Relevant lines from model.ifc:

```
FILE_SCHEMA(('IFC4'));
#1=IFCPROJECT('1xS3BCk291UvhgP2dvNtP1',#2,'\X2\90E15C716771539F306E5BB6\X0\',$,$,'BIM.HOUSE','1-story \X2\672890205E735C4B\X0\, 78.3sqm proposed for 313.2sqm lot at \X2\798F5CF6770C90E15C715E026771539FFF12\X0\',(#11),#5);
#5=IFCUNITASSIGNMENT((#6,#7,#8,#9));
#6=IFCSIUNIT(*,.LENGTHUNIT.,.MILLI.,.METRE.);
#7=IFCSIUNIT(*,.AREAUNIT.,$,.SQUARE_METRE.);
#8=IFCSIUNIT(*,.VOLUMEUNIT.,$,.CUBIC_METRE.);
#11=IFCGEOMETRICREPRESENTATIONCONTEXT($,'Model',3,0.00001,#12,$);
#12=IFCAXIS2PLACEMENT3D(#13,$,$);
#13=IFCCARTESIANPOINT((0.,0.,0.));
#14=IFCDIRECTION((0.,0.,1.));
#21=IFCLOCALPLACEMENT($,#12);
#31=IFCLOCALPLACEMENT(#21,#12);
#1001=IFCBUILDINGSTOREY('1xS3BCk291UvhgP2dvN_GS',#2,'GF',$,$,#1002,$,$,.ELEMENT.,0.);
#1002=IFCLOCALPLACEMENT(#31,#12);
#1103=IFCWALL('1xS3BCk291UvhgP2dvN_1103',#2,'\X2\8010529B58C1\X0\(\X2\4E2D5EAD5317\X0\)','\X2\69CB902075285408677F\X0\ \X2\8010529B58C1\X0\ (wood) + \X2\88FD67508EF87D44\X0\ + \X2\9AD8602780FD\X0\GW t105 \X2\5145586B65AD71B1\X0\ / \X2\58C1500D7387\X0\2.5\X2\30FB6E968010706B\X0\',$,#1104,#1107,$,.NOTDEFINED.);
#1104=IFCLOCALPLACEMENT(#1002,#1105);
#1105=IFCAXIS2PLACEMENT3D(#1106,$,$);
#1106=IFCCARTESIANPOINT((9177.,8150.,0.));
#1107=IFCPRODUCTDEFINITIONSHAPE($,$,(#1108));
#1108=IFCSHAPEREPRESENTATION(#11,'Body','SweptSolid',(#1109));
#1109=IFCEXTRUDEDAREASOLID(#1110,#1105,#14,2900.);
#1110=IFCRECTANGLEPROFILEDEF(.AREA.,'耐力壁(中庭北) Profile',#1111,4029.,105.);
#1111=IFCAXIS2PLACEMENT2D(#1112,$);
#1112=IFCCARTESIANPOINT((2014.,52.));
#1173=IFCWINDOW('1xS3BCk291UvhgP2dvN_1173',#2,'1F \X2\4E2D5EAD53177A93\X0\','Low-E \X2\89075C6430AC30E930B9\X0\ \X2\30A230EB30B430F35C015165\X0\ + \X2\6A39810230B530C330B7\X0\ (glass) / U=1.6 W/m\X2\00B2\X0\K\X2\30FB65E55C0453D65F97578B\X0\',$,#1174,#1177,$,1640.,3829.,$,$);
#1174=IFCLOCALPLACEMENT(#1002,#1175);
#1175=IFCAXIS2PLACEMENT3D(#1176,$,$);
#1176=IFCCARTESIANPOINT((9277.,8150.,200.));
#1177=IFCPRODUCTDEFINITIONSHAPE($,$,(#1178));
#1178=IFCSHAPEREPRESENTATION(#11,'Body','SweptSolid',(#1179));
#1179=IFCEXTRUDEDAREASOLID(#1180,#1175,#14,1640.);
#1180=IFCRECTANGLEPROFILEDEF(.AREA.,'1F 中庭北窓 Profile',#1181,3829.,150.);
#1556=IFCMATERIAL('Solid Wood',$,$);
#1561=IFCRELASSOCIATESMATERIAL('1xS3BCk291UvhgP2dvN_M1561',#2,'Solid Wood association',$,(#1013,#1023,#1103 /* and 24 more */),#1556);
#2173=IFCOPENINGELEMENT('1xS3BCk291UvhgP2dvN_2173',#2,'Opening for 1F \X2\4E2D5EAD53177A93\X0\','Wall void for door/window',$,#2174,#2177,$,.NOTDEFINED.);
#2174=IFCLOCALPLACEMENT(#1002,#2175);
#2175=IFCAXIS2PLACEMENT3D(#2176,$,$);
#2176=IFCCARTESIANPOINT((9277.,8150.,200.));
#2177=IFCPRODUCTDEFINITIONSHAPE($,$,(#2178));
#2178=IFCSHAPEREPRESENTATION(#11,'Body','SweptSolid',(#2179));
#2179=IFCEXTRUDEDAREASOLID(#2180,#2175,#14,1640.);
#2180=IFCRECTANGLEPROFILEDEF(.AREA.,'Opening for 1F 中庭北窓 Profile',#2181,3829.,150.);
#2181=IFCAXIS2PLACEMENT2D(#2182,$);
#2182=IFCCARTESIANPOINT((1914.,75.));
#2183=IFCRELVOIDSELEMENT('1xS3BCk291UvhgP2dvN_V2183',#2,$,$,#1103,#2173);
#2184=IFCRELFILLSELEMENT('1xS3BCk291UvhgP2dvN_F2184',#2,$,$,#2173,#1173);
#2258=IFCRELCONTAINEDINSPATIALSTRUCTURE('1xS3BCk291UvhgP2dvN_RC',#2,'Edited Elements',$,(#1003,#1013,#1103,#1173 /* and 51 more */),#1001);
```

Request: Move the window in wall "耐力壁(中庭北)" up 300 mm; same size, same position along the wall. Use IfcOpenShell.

```python
import numpy as np
import ifcopenshell
import ifcopenshell.api.geometry
import ifcopenshell.util.placement
import ifcopenshell.util.unit

model = ifcopenshell.open("model.ifc")
unit_scale = ifcopenshell.util.unit.calculate_unit_scale(model)

window = model.by_guid("1xS3BCk291UvhgP2dvN_1173")
opening = window.FillsVoids[0].RelatingOpeningElement
dz = 300.0

shift = np.array([0.0, 0.0, dz])
# The window is not placed relative to its opening, so move both.
for product in (opening, window):
    matrix = ifcopenshell.util.placement.get_local_placement(product.ObjectPlacement)
    matrix[:3, 3] += shift
    ifcopenshell.api.geometry.edit_object_placement(model, product=product, matrix=matrix, is_si=False)

print(f"moved by {dz * unit_scale:+.3f} m")

model.write("model_updated.ifc")
```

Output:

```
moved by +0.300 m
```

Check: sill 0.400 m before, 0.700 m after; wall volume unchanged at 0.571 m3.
